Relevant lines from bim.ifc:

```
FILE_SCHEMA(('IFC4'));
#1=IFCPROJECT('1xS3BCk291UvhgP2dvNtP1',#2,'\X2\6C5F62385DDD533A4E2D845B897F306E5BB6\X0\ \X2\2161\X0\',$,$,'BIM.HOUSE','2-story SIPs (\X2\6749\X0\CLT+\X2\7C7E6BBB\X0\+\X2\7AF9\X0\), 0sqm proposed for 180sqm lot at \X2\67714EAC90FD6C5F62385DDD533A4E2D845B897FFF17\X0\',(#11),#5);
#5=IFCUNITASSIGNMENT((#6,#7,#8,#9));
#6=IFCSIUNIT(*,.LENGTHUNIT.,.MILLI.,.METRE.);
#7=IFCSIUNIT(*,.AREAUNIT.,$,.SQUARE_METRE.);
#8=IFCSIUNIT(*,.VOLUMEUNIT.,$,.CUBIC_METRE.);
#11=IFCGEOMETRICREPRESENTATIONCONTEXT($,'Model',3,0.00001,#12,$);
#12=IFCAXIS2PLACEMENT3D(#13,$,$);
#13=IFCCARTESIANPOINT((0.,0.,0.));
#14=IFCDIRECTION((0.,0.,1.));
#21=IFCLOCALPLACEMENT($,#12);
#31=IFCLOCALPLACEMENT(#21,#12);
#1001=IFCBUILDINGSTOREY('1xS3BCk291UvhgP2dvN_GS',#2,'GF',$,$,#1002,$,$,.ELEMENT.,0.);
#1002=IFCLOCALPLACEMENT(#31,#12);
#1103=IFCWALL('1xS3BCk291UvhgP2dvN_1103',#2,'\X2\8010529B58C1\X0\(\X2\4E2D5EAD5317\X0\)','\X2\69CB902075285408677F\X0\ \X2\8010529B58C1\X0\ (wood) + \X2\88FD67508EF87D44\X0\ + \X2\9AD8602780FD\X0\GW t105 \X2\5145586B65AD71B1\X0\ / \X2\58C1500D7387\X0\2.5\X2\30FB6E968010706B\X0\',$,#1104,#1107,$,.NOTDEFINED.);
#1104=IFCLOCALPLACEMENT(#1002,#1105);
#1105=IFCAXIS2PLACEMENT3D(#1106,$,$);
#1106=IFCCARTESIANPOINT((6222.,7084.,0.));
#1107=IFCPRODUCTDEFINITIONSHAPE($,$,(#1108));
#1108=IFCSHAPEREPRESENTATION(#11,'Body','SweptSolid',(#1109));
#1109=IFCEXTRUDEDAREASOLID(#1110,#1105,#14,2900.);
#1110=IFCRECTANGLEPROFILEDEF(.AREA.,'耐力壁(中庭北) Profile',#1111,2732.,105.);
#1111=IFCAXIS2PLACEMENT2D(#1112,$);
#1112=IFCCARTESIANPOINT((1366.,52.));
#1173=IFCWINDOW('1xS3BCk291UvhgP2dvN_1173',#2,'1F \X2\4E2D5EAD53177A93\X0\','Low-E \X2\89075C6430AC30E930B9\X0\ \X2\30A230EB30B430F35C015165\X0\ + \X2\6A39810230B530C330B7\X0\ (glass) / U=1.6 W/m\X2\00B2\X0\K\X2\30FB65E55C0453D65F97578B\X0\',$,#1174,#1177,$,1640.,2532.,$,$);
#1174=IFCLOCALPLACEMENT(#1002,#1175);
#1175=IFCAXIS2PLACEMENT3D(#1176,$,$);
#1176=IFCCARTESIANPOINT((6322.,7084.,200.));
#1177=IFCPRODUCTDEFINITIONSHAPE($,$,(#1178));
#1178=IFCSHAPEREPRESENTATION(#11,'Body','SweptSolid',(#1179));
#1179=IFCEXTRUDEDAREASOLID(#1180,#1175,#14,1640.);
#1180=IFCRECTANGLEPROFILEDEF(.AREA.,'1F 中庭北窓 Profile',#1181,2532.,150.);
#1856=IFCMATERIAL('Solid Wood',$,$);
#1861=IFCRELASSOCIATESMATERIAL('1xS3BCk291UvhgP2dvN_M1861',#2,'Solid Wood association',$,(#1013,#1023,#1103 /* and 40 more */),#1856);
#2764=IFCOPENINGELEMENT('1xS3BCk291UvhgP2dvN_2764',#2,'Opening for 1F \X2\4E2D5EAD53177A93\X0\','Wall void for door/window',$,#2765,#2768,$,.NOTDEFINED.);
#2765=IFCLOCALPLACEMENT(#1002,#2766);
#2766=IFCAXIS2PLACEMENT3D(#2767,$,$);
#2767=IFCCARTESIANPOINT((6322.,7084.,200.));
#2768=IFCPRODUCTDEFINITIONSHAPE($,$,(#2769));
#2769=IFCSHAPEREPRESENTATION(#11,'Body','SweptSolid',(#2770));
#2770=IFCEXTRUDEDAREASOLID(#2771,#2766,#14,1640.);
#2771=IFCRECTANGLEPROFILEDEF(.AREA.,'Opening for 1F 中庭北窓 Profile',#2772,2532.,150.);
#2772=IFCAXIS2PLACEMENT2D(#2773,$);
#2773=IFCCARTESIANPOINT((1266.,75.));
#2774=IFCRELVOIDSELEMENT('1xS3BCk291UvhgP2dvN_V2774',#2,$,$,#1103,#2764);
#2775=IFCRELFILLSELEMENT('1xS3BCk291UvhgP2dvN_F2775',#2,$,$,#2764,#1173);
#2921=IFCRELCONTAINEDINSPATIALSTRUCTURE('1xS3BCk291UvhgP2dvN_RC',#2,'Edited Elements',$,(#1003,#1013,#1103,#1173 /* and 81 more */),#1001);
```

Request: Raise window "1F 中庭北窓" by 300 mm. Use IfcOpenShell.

```python
import numpy as np
import ifcopenshell
import ifcopenshell.api.geometry
import ifcopenshell.util.placement
import ifcopenshell.util.unit

model = ifcopenshell.open("bim.ifc")
unit_scale = ifcopenshell.util.unit.calculate_unit_scale(model)

window = model.by_guid("1xS3BCk291UvhgP2dvN_1173")
opening = window.FillsVoids[0].RelatingOpeningElement
dz = 0.3 / unit_scale

shift = np.array([0.0, 0.0, dz])
# The window is not placed relative to its opening, so move both.
for product in (opening, window):
    matrix = ifcopenshell.util.placement.get_local_placement(product.ObjectPlacement)
    matrix[:3, 3] += shift
    ifcopenshell.api.geometry.edit_object_placement(model, product=product, matrix=matrix, is_si=False)

print(f"moved by {dz * unit_scale:+.3f} m")

model.write("bim_edited.ifc")
```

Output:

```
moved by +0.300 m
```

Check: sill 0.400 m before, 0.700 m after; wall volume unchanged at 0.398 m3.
